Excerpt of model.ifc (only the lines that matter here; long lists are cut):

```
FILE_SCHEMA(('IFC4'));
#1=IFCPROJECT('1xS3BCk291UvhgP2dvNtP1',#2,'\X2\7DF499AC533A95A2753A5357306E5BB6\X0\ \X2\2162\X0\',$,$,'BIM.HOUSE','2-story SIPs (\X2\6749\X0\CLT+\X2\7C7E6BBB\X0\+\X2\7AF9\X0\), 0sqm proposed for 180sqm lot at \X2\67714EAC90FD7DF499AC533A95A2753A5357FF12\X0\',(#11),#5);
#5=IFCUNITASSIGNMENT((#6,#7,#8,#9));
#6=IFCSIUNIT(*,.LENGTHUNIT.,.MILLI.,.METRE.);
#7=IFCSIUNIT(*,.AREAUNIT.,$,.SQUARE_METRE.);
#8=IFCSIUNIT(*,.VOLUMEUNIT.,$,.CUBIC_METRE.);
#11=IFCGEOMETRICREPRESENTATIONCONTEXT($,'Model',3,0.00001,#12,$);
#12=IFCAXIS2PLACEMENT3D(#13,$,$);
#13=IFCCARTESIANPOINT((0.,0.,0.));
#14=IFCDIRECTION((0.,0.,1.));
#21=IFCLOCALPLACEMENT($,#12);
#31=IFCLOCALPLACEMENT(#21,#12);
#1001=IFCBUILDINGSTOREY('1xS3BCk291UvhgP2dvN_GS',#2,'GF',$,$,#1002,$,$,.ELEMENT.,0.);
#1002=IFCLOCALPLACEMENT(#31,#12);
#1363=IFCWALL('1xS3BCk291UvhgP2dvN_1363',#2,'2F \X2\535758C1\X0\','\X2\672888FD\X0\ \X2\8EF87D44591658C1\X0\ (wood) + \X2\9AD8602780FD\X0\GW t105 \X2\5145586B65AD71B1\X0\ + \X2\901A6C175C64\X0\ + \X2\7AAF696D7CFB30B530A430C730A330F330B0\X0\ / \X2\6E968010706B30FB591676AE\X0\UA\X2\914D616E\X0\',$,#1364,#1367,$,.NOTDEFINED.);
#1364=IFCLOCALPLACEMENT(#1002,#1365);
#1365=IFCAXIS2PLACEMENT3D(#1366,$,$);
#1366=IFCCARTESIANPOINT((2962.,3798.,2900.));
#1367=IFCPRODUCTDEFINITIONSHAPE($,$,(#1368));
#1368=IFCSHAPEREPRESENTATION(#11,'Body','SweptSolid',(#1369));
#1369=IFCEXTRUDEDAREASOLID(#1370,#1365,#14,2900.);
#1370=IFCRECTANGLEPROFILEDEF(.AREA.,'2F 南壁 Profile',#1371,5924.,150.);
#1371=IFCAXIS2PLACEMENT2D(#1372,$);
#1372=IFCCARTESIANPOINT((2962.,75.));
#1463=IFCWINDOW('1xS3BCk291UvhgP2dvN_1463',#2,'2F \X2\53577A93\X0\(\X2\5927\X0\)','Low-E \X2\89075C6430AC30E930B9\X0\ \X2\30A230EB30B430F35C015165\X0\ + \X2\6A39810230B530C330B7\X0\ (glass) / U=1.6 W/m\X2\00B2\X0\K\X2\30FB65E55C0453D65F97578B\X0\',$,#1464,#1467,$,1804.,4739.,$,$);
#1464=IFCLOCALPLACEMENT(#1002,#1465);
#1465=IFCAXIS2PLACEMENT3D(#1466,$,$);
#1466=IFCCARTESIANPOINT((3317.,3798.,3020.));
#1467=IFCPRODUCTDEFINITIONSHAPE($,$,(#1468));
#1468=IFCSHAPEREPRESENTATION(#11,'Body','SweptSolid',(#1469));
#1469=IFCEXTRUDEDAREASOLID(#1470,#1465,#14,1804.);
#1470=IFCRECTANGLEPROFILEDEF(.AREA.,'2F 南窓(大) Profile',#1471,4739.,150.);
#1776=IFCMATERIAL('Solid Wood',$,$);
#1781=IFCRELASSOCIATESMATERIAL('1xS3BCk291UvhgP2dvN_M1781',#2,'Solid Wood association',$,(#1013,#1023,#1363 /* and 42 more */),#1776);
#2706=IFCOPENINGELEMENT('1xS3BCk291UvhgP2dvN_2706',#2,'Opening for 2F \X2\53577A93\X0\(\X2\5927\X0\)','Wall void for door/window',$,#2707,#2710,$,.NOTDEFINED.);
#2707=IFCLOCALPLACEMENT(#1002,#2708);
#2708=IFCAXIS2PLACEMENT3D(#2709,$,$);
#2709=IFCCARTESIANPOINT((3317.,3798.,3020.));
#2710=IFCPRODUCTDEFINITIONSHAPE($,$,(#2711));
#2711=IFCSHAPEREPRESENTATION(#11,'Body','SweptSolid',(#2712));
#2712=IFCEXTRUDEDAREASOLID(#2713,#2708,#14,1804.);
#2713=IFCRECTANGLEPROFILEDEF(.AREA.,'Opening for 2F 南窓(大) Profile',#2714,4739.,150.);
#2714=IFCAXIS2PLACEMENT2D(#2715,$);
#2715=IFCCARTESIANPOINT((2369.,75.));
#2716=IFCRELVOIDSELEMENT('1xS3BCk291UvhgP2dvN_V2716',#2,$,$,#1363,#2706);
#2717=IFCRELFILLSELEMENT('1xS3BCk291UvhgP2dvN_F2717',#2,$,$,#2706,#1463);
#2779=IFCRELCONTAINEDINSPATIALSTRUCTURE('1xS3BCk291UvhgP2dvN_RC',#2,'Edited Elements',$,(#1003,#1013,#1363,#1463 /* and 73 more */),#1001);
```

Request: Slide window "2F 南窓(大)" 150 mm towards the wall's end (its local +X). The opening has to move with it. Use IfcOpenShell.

```python
import ifcopenshell
import ifcopenshell.api.geometry
import ifcopenshell.util.placement
import ifcopenshell.util.unit

model = ifcopenshell.open("model.ifc")
unit_scale = ifcopenshell.util.unit.calculate_unit_scale(model)

window = model.by_guid("1xS3BCk291UvhgP2dvN_1463")
opening = window.FillsVoids[0].RelatingOpeningElement
wall = opening.VoidsElements[0].RelatingBuildingElement

wall_matrix = ifcopenshell.util.placement.get_local_placement(wall.ObjectPlacement)
shift = wall_matrix[:3, 0] * 0.15 / unit_scale
before = ifcopenshell.util.placement.get_local_placement(window.ObjectPlacement)[:3, 3].copy()

# The window is not placed relative to its opening, so move both.
for product in (opening, window):
    matrix = ifcopenshell.util.placement.get_local_placement(product.ObjectPlacement)
    matrix[:3, 3] += shift
    ifcopenshell.api.geometry.edit_object_placement(model, product=product, matrix=matrix, is_si=False)

after = ifcopenshell.util.placement.get_local_placement(window.ObjectPlacement)[:3, 3]
print("window moved by", (after - before).round(3) + 0.0)

model.write("model_v2.ifc")
```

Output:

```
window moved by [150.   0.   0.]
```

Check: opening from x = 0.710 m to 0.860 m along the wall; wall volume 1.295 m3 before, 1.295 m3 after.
